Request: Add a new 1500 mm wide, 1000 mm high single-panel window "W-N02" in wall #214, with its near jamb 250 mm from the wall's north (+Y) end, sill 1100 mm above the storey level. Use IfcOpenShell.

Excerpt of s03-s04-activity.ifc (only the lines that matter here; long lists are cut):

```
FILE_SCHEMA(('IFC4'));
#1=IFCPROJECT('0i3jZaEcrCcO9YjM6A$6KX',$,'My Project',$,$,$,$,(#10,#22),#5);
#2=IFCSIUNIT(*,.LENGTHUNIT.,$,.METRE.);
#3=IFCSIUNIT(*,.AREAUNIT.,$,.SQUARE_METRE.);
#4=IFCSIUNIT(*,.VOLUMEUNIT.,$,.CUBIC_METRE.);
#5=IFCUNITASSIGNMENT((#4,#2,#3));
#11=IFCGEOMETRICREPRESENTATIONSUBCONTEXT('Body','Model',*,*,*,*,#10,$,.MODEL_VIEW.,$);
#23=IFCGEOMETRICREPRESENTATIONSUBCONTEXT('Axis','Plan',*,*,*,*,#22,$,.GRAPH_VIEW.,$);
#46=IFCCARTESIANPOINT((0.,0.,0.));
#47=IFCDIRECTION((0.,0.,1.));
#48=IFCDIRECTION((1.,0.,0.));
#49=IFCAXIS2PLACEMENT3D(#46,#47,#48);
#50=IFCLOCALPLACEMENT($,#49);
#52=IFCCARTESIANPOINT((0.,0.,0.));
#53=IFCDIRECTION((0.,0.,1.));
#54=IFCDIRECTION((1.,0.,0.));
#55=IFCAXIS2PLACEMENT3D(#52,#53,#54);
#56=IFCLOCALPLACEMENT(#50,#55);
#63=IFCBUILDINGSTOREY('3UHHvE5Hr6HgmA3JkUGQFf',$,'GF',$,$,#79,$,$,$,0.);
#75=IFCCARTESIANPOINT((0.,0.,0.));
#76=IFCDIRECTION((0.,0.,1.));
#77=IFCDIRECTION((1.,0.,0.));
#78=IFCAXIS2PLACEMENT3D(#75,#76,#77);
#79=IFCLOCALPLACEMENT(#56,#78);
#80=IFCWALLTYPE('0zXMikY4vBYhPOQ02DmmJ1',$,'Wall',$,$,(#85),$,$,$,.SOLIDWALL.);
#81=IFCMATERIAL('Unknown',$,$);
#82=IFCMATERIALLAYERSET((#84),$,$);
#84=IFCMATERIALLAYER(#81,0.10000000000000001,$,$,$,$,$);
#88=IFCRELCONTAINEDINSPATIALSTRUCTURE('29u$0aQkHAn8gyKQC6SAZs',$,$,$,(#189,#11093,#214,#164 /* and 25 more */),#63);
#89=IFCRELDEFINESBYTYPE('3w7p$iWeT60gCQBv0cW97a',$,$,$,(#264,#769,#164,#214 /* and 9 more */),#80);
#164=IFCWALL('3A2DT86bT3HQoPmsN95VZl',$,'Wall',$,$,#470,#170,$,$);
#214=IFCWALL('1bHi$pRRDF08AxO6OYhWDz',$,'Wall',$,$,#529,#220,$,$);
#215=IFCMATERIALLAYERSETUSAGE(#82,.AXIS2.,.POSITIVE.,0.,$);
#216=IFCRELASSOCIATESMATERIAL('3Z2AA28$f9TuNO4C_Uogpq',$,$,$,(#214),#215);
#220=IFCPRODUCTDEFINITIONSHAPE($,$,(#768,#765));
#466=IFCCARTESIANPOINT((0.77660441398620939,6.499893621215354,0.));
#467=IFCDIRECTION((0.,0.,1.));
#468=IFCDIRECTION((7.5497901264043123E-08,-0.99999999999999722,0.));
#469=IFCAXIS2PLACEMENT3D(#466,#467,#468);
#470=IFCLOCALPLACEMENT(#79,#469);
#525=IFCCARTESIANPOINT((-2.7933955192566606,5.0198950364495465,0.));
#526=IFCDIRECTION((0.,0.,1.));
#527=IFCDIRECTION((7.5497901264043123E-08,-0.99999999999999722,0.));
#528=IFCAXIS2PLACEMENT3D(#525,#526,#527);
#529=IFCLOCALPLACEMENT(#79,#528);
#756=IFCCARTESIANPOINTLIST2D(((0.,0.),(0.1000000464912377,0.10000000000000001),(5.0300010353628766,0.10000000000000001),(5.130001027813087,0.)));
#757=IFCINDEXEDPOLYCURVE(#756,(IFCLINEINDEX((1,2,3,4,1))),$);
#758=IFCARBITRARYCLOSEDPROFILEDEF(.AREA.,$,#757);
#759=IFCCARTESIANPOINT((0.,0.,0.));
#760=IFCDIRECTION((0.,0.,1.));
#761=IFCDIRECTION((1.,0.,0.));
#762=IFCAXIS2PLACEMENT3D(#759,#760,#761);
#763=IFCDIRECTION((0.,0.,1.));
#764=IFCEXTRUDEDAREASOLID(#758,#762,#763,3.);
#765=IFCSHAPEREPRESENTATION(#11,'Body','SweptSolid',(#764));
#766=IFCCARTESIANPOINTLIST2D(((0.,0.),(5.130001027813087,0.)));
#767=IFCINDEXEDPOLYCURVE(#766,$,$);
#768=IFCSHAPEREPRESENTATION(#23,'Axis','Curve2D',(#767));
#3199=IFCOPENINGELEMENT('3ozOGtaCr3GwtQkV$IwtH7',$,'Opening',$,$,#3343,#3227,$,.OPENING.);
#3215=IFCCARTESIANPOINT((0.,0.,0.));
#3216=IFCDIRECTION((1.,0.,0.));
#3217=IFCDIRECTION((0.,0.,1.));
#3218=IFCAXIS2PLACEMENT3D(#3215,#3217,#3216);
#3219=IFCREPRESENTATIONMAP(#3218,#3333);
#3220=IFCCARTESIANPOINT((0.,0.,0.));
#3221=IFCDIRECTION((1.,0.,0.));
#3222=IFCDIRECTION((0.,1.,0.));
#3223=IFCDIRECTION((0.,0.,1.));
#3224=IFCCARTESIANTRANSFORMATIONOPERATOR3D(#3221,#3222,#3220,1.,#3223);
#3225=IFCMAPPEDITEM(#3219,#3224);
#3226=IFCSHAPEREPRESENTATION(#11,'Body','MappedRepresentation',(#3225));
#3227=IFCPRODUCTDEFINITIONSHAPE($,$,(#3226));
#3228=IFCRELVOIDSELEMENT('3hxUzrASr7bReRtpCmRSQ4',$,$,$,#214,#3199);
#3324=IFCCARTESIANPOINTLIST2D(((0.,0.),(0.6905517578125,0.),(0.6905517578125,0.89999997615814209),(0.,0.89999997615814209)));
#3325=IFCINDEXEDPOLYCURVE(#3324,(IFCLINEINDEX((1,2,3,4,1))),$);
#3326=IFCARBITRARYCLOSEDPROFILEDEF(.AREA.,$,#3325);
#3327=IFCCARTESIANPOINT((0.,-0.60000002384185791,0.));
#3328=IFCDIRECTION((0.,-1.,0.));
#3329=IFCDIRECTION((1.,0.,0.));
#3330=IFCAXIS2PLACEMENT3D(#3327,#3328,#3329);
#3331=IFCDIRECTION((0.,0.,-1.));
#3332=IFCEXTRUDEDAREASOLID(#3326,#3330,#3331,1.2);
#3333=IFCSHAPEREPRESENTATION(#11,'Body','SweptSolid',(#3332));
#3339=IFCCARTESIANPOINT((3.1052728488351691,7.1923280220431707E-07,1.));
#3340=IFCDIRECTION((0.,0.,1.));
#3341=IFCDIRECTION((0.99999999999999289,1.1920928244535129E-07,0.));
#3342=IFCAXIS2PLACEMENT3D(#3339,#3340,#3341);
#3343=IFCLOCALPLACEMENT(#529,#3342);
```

```python
import numpy as np
import ifcopenshell
import ifcopenshell.api.feature
import ifcopenshell.api.geometry
import ifcopenshell.api.root
import ifcopenshell.api.spatial
import ifcopenshell.geom
import ifcopenshell.util.element
import ifcopenshell.util.placement
import ifcopenshell.util.representation
import ifcopenshell.util.shape
import ifcopenshell.util.unit

model = ifcopenshell.open("s03-s04-activity.ifc")
unit_scale = ifcopenshell.util.unit.calculate_unit_scale(model)
settings = ifcopenshell.geom.settings()


def volume(element):
    """Net volume in cubic metres, openings subtracted."""
    shape = ifcopenshell.geom.create_shape(settings, element)
    return ifcopenshell.util.shape.get_volume(shape.geometry)


wall = model.by_id(214)
storey = ifcopenshell.util.element.get_container(wall, ifc_class="IfcBuildingStorey")
context = ifcopenshell.util.representation.get_context(model, "Model", "Body", "MODEL_VIEW")
before = volume(wall)

width, height, from_end, sill = 1.5, 1, 0.25, 1.1  # metres

# The wall runs along its own X axis, and the end named is its -X end.
wall_shape = ifcopenshell.geom.create_shape(settings, wall)
x, y, z = ifcopenshell.util.shape.get_vertices(wall_shape.geometry).T
start = x.min() + from_end
face, thickness = float(y.min()), float(y.max() - y.min())
wall_matrix = ifcopenshell.util.placement.get_local_placement(wall.ObjectPlacement)
level = ifcopenshell.util.placement.get_local_placement(storey.ObjectPlacement)[2, 3]


def in_wall(x, y):
    """Placement at x, y metres in the wall's axes, at sill height."""
    matrix = wall_matrix.copy()
    matrix[:, 3] = wall_matrix @ np.array([x / unit_scale, y / unit_scale, 0.0, 1.0])
    matrix[2, 3] = level + sill / unit_scale
    return matrix


# Opening: a box that overshoots both wall faces by 50 mm.
opening = ifcopenshell.api.root.create_entity(model, ifc_class="IfcOpeningElement", predefined_type="OPENING")
box = ifcopenshell.api.geometry.add_wall_representation(
    model, context=context, length=width, height=height, thickness=thickness + 0.1
)
ifcopenshell.api.geometry.assign_representation(model, product=opening, representation=box)
ifcopenshell.api.geometry.edit_object_placement(model, product=opening, matrix=in_wall(start, face - 0.05), is_si=False)
ifcopenshell.api.feature.add_feature(model, feature=opening, element=wall)

window = ifcopenshell.api.root.create_entity(model, ifc_class="IfcWindow", name="W-N02", predefined_type="WINDOW")
window.OverallWidth, window.OverallHeight = width / unit_scale, height / unit_scale
window.PartitioningType = "SINGLE_PANEL"
body = ifcopenshell.api.geometry.add_window_representation(
    model,
    context=context,
    overall_width=window.OverallWidth,
    overall_height=window.OverallHeight,
    partition_type="SINGLE_PANEL",
)
ifcopenshell.api.geometry.assign_representation(model, product=window, representation=body)
ifcopenshell.api.spatial.assign_container(model, products=[window], relating_structure=storey)
ifcopenshell.api.feature.add_filling(model, opening=opening, element=window)

# Centre the window in the wall's thickness.
ifcopenshell.api.geometry.edit_object_placement(model, product=window, matrix=in_wall(start, face), is_si=False)
window_shape = ifcopenshell.geom.create_shape(settings, window)
depth = ifcopenshell.util.shape.get_vertices(window_shape.geometry)[:, 1]
offset = face + thickness / 2 - (depth.min() + depth.max()) / 2
ifcopenshell.api.geometry.edit_object_placement(model, product=window, matrix=in_wall(start, offset), is_si=False)

after = volume(wall)

print(f"wall volume {before:.3f} -> {after:.3f} m3")

model.write("s03-s04-activity_rev.ifc")
```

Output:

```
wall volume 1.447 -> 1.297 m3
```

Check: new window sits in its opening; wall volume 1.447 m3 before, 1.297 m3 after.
